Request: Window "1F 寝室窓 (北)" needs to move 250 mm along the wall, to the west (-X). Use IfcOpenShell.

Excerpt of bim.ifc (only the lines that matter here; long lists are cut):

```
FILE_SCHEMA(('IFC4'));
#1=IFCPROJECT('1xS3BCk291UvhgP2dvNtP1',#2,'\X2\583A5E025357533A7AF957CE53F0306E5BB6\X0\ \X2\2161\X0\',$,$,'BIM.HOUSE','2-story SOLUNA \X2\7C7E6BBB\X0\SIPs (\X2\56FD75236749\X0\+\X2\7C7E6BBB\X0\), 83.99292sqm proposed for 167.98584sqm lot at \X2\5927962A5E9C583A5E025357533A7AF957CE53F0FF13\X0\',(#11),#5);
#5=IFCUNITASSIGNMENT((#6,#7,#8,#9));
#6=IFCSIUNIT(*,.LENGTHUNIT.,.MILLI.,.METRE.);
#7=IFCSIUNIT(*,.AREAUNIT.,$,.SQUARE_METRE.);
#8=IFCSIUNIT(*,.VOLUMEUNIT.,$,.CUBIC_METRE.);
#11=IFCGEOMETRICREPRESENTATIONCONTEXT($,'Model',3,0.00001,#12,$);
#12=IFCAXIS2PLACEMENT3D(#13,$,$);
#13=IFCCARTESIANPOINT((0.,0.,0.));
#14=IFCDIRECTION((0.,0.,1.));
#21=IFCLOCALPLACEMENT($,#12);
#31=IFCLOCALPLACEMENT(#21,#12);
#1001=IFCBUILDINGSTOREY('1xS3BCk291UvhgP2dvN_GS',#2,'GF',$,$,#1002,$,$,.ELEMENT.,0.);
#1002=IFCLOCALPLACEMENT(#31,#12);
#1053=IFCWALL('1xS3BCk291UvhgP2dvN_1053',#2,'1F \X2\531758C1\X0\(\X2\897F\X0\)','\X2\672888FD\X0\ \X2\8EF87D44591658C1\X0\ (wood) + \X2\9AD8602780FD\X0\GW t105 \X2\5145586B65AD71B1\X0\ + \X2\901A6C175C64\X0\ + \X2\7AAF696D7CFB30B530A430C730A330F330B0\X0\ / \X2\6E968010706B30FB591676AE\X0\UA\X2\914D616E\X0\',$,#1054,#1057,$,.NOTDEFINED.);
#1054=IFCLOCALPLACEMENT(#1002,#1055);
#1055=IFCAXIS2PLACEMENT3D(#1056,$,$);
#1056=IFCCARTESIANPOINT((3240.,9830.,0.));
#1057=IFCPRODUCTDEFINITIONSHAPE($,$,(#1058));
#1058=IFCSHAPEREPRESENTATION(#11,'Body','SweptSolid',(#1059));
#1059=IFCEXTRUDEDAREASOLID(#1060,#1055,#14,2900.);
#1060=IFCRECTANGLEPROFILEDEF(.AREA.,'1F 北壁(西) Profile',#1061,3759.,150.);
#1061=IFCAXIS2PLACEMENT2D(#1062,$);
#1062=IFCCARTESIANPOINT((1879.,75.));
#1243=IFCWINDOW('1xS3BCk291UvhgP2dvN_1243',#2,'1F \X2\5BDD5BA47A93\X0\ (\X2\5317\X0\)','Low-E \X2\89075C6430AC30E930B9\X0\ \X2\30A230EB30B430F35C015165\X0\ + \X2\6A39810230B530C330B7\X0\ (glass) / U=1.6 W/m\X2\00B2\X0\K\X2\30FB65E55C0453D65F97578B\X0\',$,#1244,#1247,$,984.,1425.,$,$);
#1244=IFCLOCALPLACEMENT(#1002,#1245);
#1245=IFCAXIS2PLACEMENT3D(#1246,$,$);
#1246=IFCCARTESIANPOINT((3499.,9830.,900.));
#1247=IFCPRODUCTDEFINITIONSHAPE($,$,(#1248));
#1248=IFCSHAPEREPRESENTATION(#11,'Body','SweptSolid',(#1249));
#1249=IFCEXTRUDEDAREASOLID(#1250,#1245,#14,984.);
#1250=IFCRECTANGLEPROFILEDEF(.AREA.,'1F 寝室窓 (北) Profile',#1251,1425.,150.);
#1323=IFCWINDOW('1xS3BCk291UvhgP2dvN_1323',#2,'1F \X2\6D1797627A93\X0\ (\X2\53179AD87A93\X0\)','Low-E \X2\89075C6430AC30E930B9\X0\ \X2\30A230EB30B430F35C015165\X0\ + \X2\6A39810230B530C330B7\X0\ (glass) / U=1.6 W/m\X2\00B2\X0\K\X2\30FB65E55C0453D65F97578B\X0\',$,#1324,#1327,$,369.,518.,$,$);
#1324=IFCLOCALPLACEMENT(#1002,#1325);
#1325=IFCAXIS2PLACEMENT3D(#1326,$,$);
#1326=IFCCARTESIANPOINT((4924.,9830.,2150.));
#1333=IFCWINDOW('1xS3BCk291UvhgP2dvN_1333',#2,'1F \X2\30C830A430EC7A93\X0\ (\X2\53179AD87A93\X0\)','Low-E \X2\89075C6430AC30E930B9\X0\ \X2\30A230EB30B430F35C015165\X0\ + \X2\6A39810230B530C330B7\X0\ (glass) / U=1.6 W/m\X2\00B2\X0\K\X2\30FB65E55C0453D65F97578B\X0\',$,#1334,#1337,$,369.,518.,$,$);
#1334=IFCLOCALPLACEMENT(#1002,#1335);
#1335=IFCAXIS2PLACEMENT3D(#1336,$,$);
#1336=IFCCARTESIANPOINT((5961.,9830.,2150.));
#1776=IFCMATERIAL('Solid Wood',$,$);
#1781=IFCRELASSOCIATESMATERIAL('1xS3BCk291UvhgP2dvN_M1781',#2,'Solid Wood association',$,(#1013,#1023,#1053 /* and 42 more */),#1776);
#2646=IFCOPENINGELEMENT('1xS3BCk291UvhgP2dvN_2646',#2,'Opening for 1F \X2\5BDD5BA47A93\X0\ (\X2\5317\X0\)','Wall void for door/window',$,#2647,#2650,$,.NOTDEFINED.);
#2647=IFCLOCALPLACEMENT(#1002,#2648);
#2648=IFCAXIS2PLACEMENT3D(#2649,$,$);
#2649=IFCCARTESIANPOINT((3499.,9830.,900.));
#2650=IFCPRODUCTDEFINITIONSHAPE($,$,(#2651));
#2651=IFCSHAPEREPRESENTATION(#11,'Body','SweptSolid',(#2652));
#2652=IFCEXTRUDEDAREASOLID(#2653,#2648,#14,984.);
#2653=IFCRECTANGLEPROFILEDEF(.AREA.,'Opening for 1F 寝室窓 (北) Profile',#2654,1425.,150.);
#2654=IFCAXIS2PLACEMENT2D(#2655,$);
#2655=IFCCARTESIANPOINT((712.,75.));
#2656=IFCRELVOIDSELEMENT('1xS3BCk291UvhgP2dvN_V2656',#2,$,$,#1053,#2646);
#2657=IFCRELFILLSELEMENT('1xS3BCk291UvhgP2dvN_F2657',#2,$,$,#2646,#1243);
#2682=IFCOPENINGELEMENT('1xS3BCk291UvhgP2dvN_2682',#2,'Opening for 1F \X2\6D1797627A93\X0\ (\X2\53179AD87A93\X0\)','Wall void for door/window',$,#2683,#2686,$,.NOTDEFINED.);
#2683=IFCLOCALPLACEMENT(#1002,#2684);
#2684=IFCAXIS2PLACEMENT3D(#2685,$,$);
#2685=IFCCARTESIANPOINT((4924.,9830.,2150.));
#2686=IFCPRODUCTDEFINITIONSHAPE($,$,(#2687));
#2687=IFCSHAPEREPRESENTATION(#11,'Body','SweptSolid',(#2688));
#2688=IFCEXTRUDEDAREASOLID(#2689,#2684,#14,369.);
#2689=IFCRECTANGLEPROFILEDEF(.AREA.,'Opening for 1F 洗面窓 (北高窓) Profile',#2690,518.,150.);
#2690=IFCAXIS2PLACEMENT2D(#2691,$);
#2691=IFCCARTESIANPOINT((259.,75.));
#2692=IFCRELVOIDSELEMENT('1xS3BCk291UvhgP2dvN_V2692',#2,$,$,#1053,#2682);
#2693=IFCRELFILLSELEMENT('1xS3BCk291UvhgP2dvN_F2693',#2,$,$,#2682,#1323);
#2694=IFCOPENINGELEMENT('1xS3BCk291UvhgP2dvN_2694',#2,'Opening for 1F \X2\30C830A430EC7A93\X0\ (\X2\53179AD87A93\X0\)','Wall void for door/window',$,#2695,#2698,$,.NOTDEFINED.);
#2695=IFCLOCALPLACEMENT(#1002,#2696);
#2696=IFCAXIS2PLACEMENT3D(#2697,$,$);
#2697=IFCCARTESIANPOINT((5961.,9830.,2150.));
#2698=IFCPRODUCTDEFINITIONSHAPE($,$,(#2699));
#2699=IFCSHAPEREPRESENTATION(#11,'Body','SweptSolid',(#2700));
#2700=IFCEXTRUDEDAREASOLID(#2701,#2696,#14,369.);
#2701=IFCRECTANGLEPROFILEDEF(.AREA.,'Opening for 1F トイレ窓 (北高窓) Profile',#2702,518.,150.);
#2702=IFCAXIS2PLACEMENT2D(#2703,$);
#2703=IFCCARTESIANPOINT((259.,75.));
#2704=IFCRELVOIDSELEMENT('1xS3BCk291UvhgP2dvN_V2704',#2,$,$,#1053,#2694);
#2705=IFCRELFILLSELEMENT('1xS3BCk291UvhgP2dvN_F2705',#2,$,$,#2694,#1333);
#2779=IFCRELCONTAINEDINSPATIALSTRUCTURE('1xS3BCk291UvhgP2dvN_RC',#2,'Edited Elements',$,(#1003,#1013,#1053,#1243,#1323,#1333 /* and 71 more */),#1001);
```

```python
import ifcopenshell
import ifcopenshell.api.geometry
import ifcopenshell.util.placement

model = ifcopenshell.open("bim.ifc")

window = model.by_guid("1xS3BCk291UvhgP2dvN_1243")
opening = window.FillsVoids[0].RelatingOpeningElement
wall = opening.VoidsElements[0].RelatingBuildingElement

wall_matrix = ifcopenshell.util.placement.get_local_placement(wall.ObjectPlacement)
shift = wall_matrix[:3, 0] * -250.0
before = ifcopenshell.util.placement.get_local_placement(window.ObjectPlacement)[:3, 3].copy()

# The window is not placed relative to its opening, so move both.
for product in (opening, window):
    matrix = ifcopenshell.util.placement.get_local_placement(product.ObjectPlacement)
    matrix[:3, 3] += shift
    ifcopenshell.api.geometry.edit_object_placement(model, product=product, matrix=matrix, is_si=False)

after = ifcopenshell.util.placement.get_local_placement(window.ObjectPlacement)[:3, 3]
print("window moved by", (after - before).round(3) + 0.0)

model.write("bim_updated.ifc")
```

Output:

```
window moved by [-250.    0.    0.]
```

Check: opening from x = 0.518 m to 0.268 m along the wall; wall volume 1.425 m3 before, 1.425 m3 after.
